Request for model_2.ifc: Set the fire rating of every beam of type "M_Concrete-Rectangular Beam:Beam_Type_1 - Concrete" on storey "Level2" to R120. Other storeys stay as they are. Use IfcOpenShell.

First a look at what the model holds.

```python
import ifcopenshell
import ifcopenshell.util.element

model = ifcopenshell.open("model_2.ifc")
print(model.schema)
storey = next(s for s in model.by_type("IfcBuildingStorey") if s.Name == "Level2")
beams = [e for e in ifcopenshell.util.element.get_decomposition(storey) if e.is_a("IfcBeam")]
seen = {}
for e in beams:
    element_type = ifcopenshell.util.element.get_type(e)
    key = (element_type.Name if element_type != e and element_type else None, ifcopenshell.util.element.get_pset(e, "Pset_BeamCommon", "FireRating"))
    seen[key] = seen.get(key, 0) + 1
for (name, value), count in sorted(seen.items(), key=str):
    print(count, "x", name, "|", value)
```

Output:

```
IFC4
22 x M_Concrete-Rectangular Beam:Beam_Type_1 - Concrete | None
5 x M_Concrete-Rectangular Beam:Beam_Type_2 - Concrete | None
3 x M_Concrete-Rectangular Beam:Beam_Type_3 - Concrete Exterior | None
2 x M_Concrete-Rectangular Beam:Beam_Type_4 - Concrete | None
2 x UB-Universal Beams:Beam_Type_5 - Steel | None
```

```python
import ifcopenshell
import ifcopenshell.api.pset
import ifcopenshell.util.element

model = ifcopenshell.open("model_2.ifc")

storey = next(s for s in model.by_type("IfcBuildingStorey") if s.Name == "Level2")
beams = [e for e in ifcopenshell.util.element.get_decomposition(storey) if e.is_a("IfcBeam")]

count = 0
for e in beams:
    element_type = ifcopenshell.util.element.get_type(e)
    if element_type in (None, e) or element_type.Name != "M_Concrete-Rectangular Beam:Beam_Type_1 - Concrete":
        continue
    # add_pset returns the element's existing set when there is one.
    pset = ifcopenshell.api.pset.add_pset(model, product=e, name="Pset_BeamCommon")
    ifcopenshell.api.pset.edit_pset(model, pset=pset, properties={"FireRating": "R120"})
    count += 1

print(count, "beams updated")

model.write("model_2_updated.ifc")
```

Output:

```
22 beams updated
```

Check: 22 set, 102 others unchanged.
